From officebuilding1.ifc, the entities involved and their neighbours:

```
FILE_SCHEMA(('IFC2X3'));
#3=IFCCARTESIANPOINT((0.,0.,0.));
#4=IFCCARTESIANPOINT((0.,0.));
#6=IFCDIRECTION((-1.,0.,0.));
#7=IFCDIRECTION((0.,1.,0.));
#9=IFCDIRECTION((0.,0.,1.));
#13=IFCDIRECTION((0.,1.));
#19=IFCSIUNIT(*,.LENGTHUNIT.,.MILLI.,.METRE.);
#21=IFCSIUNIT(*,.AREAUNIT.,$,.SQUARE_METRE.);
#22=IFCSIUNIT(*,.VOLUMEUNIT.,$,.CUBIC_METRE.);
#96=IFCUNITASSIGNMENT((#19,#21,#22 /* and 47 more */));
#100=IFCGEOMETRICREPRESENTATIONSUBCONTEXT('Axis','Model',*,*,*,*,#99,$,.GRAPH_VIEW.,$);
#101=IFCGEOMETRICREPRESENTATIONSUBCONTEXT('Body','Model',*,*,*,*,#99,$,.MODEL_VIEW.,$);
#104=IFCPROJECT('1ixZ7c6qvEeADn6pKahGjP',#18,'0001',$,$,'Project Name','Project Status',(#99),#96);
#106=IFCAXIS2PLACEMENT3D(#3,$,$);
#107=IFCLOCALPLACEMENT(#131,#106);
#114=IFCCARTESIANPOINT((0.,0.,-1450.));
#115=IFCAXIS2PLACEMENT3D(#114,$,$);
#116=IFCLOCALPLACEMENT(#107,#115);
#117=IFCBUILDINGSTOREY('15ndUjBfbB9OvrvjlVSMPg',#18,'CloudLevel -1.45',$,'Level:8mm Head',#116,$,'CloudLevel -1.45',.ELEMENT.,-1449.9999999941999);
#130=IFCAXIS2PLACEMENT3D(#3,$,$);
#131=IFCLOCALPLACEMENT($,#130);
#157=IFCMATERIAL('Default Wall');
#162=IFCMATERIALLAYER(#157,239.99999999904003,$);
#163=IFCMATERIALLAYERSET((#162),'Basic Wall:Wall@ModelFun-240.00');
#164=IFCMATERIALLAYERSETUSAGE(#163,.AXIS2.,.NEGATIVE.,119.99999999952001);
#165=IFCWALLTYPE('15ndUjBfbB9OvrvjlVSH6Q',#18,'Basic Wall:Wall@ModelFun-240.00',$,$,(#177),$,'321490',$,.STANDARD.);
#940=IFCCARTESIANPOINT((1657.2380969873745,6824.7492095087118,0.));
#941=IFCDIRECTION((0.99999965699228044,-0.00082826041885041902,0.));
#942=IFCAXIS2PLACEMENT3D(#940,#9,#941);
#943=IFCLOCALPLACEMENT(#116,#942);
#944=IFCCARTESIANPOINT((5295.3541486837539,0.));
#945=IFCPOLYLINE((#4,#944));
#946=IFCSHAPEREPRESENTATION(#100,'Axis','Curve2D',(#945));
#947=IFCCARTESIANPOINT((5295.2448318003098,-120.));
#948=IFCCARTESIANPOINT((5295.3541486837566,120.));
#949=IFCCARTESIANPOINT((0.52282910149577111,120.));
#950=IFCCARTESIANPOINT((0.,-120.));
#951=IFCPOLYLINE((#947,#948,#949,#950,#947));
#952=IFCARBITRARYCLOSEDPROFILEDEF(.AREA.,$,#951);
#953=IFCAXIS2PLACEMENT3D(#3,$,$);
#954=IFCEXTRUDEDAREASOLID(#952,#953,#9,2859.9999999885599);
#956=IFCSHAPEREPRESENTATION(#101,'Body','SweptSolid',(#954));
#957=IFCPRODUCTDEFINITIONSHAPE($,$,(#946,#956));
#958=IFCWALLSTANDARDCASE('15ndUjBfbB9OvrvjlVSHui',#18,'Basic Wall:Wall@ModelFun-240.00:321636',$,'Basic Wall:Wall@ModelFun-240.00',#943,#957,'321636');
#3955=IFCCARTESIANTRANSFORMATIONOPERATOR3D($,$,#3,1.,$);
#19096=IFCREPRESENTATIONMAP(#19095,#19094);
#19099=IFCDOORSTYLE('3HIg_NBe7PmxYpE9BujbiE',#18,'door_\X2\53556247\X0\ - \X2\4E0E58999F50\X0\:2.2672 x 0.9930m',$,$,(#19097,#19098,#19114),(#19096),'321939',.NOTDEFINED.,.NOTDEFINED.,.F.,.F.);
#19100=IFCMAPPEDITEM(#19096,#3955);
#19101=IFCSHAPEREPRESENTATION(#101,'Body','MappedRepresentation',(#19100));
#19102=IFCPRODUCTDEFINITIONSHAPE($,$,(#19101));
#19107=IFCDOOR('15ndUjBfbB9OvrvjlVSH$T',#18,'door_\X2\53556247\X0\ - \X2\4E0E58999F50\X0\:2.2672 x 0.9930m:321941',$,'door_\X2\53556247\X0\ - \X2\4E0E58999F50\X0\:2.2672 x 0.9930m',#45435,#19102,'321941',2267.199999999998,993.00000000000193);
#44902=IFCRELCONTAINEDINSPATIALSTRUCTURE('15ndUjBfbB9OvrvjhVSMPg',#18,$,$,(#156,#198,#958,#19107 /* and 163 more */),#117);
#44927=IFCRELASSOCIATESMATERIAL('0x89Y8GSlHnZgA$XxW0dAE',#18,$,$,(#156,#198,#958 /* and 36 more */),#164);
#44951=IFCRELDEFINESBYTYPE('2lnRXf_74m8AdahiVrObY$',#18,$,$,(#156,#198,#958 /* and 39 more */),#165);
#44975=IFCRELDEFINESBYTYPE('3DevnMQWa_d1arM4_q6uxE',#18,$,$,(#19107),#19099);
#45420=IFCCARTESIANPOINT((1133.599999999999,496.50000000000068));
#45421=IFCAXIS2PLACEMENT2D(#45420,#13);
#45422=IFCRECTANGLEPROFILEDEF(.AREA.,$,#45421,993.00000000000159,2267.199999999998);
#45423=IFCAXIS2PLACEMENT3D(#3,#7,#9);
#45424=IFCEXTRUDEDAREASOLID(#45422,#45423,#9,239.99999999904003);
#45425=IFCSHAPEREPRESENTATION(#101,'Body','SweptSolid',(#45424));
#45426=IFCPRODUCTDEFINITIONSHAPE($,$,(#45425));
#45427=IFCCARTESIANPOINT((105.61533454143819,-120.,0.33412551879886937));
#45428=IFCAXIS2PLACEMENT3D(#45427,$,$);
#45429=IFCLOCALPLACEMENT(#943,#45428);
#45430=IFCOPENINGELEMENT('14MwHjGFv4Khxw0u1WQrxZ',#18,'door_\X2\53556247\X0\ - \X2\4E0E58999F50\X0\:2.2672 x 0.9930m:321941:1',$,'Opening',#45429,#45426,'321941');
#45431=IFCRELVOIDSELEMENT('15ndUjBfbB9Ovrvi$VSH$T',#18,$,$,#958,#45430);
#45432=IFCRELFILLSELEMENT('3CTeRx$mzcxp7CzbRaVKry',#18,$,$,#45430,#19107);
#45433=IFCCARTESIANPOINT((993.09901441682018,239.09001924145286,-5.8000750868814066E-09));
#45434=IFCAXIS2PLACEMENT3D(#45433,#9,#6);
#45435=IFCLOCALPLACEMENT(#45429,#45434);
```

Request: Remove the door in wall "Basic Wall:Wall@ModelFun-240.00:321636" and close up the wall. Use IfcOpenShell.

```python
import ifcopenshell
import ifcopenshell.api.feature
import ifcopenshell.api.root
import ifcopenshell.geom
import ifcopenshell.util.shape

model = ifcopenshell.open("officebuilding1.ifc")
settings = ifcopenshell.geom.settings()


def volume(element):
    """Net volume in cubic metres, openings subtracted."""
    shape = ifcopenshell.geom.create_shape(settings, element)
    return ifcopenshell.util.shape.get_volume(shape.geometry)


door = model.by_guid("15ndUjBfbB9OvrvjlVSH$T")
opening = door.FillsVoids[0].RelatingOpeningElement
wall = opening.VoidsElements[0].RelatingBuildingElement
before = volume(wall)

ifcopenshell.api.root.remove_product(model, product=door)
ifcopenshell.api.feature.remove_feature(model, feature=opening)

after = volume(wall)

print(f"wall volume {before:.3f} -> {after:.3f} m3")

model.write("officebuilding1_v2.ifc")
```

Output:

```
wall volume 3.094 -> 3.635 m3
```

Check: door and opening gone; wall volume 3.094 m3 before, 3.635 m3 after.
